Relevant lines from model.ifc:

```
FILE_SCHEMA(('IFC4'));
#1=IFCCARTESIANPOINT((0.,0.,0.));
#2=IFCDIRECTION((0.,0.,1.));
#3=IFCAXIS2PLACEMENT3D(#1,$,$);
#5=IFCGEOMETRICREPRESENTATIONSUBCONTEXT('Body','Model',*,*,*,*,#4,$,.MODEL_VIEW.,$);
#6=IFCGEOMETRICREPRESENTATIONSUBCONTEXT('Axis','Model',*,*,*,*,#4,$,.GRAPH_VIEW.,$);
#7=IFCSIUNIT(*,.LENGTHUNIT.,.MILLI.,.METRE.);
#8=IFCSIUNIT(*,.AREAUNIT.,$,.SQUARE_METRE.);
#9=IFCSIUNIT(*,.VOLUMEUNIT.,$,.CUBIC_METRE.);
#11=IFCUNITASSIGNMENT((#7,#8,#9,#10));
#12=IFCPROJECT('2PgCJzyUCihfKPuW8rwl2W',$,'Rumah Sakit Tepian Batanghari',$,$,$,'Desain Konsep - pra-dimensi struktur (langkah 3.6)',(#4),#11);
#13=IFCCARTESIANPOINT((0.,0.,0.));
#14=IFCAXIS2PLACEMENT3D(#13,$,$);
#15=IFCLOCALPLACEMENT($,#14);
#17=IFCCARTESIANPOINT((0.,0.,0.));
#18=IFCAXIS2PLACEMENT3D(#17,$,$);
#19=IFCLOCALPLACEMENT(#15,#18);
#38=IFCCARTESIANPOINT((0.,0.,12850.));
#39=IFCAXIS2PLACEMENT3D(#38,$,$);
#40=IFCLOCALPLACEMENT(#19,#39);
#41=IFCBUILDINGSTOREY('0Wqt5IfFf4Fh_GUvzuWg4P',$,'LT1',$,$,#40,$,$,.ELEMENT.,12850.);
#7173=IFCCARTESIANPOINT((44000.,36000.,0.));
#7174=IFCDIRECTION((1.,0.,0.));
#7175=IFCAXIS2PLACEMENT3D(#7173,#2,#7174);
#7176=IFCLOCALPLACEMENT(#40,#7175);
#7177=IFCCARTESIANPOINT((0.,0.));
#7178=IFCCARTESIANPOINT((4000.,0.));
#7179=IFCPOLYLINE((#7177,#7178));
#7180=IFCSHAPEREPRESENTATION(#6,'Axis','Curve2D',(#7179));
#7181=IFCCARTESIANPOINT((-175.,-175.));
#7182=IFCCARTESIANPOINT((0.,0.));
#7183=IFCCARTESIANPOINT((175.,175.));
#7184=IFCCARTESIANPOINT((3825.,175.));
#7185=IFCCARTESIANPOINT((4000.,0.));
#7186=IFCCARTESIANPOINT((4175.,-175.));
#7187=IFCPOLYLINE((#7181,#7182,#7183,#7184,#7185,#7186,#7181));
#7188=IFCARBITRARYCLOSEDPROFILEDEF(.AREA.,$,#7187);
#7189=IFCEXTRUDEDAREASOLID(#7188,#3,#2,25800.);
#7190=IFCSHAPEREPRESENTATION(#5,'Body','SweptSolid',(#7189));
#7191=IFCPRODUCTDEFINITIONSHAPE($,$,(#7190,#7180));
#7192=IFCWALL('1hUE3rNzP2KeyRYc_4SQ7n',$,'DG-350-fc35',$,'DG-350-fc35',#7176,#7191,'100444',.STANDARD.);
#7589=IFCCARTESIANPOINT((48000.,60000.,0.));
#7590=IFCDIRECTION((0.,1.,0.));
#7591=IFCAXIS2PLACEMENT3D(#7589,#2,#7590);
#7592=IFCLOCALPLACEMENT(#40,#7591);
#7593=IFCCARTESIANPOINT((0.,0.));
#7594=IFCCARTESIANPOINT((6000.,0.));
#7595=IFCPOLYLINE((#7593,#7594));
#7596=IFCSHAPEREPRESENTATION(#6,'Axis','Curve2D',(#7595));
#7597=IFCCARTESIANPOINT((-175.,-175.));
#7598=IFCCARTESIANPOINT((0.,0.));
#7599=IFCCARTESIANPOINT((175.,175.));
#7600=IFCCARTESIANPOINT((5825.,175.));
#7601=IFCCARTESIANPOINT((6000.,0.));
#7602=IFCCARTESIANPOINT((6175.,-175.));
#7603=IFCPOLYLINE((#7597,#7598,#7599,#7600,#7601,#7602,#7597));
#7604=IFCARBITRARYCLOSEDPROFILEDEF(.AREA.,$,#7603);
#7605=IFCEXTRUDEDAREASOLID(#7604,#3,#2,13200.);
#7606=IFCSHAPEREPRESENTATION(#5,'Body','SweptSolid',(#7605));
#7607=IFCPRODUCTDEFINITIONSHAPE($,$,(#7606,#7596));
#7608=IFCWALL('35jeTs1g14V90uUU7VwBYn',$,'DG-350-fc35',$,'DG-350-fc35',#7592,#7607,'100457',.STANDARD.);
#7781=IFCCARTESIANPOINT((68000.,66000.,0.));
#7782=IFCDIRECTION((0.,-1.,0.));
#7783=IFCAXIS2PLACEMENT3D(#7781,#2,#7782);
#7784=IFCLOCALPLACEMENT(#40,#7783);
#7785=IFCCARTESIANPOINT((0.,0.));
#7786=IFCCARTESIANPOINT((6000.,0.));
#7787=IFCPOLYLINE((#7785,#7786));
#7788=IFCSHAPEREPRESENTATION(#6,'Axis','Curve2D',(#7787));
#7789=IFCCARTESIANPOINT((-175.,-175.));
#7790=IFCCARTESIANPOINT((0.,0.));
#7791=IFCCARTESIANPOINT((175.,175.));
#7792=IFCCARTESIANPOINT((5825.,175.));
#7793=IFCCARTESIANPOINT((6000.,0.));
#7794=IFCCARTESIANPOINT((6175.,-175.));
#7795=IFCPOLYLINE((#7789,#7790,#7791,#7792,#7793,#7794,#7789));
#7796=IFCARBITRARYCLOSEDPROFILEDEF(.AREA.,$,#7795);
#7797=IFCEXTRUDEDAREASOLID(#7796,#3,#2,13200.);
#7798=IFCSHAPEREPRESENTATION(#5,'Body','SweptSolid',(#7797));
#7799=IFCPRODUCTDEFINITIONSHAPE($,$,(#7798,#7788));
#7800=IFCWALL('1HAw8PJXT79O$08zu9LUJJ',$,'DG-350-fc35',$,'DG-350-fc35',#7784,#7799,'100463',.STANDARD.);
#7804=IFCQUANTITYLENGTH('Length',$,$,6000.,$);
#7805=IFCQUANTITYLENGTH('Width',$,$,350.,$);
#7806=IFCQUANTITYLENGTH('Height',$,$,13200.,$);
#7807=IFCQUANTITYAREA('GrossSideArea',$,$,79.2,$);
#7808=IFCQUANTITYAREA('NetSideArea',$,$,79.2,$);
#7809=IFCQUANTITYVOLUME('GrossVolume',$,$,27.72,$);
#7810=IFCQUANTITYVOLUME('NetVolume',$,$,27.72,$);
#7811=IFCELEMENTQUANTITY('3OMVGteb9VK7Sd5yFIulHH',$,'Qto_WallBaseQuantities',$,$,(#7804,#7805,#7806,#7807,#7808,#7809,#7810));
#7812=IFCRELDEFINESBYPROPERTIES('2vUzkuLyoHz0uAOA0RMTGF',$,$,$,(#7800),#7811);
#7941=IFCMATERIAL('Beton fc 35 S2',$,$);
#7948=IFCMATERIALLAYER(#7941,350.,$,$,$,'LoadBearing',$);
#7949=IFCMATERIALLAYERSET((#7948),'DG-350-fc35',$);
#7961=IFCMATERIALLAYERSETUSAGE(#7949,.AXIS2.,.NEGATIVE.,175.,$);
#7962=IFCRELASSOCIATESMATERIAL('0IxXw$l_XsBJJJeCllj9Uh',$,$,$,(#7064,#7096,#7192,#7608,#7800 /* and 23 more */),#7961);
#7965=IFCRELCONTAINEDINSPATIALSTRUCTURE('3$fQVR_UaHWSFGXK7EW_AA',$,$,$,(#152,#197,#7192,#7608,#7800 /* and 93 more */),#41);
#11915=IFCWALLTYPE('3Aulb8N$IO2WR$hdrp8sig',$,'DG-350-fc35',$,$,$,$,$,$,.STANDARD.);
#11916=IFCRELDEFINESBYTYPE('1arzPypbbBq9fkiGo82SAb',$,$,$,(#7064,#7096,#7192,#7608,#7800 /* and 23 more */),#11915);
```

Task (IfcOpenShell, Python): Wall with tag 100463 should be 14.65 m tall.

```python
import ifcopenshell
import ifcopenshell.api.pset
import ifcopenshell.geom
import ifcopenshell.util.element
import ifcopenshell.util.representation
import ifcopenshell.util.shape
import ifcopenshell.util.unit

model = ifcopenshell.open("model.ifc")
unit_scale = ifcopenshell.util.unit.calculate_unit_scale(model)
area_scale = ifcopenshell.util.unit.calculate_unit_scale(model, "AREAUNIT")
volume_scale = ifcopenshell.util.unit.calculate_unit_scale(model, "VOLUMEUNIT")
settings = ifcopenshell.geom.settings()


def volume(element):
    """Net volume in cubic metres, openings subtracted."""
    shape = ifcopenshell.geom.create_shape(settings, element)
    return ifcopenshell.util.shape.get_volume(shape.geometry)


wall = model.by_id(7800)
before = volume(wall)

body = ifcopenshell.util.representation.get_representation(wall, "Model", "Body")
solid = body.Items[0]
old_height = solid.Depth
solid.Depth = 14.65 / unit_scale
after = volume(wall)
thickness = 0.35  # wall thickness in metres

# Update the stored height, areas and volumes.
qto = model.by_id(ifcopenshell.util.element.get_pset(wall, "Qto_WallBaseQuantities", should_inherit=False)["id"])
ifcopenshell.api.pset.edit_qto(model, qto=qto, properties={
    "Height": solid.Depth,
    "GrossSideArea": ifcopenshell.util.element.get_pset(wall, "Qto_WallBaseQuantities", "GrossSideArea") * solid.Depth / old_height,
    "NetSideArea": after / thickness / area_scale,
    "GrossVolume": ifcopenshell.util.element.get_pset(wall, "Qto_WallBaseQuantities", "GrossVolume") * solid.Depth / old_height,
    "NetVolume": after / volume_scale,
})

print(f"height {old_height:g} -> {solid.Depth:g}, volume {before:.3f} -> {after:.3f} m3")

model.write("model_updated.ifc")
```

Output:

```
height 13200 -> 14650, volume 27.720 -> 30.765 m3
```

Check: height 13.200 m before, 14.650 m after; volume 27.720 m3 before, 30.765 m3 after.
